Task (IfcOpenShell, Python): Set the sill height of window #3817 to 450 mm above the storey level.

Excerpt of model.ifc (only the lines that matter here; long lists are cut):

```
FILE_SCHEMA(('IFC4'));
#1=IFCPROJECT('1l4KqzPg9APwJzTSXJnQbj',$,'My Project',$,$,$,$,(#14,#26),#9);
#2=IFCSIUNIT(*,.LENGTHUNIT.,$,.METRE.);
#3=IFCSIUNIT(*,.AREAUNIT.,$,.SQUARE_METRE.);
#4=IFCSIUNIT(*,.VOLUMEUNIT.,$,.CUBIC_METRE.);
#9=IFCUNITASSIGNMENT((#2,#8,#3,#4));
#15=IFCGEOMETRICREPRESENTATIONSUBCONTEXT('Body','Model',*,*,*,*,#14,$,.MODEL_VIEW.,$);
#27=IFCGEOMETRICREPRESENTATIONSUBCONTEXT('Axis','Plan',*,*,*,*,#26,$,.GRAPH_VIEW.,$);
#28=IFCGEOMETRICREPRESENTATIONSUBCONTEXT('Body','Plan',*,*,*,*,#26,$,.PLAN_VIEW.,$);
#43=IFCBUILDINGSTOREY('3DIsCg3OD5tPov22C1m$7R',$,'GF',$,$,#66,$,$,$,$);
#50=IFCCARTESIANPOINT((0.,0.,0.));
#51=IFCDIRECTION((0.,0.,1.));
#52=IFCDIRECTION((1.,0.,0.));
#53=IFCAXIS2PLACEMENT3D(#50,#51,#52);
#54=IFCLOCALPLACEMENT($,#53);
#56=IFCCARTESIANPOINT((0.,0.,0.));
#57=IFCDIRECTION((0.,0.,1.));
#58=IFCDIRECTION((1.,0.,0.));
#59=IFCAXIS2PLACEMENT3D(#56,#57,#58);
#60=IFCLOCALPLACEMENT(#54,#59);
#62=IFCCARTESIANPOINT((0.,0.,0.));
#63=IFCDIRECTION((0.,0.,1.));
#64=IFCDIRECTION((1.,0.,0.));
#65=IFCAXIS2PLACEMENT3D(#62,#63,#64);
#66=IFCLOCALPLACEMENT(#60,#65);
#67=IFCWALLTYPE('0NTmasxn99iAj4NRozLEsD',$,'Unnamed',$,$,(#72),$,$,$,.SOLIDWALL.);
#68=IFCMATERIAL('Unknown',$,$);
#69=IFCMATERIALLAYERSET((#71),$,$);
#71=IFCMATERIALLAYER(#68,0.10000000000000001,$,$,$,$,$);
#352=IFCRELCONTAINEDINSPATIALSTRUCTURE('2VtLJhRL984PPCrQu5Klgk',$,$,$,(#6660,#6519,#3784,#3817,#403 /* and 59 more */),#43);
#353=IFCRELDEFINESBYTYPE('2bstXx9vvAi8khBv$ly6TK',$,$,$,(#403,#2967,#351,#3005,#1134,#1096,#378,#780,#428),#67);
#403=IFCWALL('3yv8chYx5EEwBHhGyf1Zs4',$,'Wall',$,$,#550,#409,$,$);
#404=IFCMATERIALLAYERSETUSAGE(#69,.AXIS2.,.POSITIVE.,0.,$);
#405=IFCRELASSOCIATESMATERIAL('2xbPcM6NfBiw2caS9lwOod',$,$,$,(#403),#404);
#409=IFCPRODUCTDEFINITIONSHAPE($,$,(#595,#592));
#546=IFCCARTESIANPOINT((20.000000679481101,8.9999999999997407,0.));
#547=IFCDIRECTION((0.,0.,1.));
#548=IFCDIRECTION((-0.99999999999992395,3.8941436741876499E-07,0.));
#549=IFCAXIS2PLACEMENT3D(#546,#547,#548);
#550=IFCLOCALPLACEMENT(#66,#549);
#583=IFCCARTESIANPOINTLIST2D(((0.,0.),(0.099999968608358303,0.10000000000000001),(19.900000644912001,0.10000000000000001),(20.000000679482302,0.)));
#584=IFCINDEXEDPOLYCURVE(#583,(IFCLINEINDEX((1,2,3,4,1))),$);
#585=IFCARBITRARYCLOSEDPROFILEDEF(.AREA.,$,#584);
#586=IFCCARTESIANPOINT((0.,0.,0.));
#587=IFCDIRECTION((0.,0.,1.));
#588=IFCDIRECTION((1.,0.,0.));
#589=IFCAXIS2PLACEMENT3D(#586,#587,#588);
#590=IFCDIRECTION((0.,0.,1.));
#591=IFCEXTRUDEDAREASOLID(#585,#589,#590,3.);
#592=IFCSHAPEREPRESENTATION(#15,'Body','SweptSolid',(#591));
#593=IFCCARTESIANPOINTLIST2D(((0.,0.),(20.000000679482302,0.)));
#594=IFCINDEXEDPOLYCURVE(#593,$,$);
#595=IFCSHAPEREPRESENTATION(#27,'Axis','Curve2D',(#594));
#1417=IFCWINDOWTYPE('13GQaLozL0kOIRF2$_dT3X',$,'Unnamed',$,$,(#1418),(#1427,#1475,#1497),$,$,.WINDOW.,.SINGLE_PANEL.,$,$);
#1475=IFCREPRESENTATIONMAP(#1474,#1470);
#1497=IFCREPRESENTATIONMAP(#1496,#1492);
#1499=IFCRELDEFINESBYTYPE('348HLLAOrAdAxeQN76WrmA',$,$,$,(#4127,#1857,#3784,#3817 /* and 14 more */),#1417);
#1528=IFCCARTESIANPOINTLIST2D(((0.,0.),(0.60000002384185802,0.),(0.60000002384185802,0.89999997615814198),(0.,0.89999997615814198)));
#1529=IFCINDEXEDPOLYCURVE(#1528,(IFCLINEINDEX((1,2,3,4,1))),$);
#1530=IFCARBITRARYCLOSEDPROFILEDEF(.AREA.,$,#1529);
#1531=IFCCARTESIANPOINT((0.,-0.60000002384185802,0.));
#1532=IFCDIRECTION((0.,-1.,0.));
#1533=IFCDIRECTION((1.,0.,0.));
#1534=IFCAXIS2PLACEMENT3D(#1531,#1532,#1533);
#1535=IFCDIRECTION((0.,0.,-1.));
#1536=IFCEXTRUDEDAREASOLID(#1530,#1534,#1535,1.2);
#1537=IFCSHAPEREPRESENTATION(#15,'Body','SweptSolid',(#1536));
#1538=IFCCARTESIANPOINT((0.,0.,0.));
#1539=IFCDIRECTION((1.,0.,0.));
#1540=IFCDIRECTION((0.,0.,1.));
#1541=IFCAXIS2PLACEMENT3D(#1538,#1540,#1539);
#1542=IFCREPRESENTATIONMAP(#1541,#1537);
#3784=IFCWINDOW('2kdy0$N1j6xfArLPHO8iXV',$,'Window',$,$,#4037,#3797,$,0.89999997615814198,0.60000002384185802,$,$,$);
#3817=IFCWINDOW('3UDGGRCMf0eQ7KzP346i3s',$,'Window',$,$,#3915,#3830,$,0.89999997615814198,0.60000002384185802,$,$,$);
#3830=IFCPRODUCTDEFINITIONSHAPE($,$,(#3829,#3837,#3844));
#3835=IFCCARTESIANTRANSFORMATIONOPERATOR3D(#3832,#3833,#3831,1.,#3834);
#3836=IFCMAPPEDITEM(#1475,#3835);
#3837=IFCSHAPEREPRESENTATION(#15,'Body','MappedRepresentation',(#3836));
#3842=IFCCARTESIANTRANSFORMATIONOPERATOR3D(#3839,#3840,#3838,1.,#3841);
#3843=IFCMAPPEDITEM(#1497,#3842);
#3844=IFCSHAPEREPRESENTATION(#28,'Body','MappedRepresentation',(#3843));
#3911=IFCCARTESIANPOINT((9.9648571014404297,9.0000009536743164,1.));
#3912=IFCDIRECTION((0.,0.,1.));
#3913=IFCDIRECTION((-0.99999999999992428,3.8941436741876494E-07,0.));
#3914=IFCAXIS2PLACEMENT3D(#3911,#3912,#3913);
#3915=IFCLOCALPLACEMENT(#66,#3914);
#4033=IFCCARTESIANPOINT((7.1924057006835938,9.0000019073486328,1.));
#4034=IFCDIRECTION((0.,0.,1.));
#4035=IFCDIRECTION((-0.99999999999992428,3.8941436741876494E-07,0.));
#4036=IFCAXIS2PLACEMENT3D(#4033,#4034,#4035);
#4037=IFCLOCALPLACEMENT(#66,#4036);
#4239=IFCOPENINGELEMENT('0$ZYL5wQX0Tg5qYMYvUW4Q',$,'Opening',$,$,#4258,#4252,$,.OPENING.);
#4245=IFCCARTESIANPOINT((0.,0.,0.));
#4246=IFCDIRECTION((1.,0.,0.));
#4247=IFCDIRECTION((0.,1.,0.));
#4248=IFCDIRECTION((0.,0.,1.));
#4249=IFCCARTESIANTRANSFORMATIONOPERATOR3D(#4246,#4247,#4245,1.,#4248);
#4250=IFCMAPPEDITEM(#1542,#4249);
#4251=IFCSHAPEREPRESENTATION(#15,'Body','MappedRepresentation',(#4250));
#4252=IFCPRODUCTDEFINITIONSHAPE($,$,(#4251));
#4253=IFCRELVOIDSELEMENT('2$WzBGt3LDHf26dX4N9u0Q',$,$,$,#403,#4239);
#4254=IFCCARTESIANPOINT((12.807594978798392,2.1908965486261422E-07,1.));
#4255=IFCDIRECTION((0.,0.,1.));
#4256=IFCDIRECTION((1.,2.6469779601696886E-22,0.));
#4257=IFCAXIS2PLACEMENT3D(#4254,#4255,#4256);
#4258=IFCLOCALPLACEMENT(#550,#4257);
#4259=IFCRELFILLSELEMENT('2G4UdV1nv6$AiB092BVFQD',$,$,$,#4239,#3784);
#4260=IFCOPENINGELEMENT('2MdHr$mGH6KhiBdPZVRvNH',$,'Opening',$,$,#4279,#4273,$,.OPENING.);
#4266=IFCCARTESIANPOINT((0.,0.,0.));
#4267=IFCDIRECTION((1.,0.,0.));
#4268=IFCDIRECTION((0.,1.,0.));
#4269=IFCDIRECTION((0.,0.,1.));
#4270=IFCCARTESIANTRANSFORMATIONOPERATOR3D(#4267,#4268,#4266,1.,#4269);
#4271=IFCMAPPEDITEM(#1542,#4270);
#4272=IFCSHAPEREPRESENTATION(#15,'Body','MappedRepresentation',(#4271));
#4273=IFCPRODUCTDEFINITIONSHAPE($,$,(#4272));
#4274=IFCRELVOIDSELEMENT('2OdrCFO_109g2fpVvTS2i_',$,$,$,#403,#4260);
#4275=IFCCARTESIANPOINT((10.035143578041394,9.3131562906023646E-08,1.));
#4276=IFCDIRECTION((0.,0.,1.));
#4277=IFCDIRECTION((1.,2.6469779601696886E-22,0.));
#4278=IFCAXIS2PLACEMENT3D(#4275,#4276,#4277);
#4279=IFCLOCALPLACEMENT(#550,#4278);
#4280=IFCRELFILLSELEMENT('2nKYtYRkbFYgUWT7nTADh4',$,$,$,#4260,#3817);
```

```python
import numpy as np
import ifcopenshell
import ifcopenshell.api.geometry
import ifcopenshell.geom
import ifcopenshell.util.element
import ifcopenshell.util.placement
import ifcopenshell.util.shape
import ifcopenshell.util.unit

model = ifcopenshell.open("model.ifc")
unit_scale = ifcopenshell.util.unit.calculate_unit_scale(model)

window = model.by_guid("3UDGGRCMf0eQ7KzP346i3s")
opening = window.FillsVoids[0].RelatingOpeningElement
storey = ifcopenshell.util.element.get_container(window, ifc_class="IfcBuildingStorey")
level = ifcopenshell.util.placement.get_local_placement(storey.ObjectPlacement)[2, 3]

# The opening's origin need not be at the sill, so measure its lowest point.
shape = ifcopenshell.geom.create_shape(ifcopenshell.geom.settings(), opening)
bottom = ifcopenshell.util.shape.get_shape_bottom_elevation(shape, shape.geometry) / unit_scale
dz = level + 0.45 / unit_scale - bottom

shift = np.array([0.0, 0.0, dz])
# The window is not placed relative to its opening, so move both.
for product in (opening, window):
    matrix = ifcopenshell.util.placement.get_local_placement(product.ObjectPlacement)
    matrix[:3, 3] += shift
    ifcopenshell.api.geometry.edit_object_placement(model, product=product, matrix=matrix, is_si=False)

print(f"moved by {dz * unit_scale:+.3f} m")

model.write("model_rev.ifc")
```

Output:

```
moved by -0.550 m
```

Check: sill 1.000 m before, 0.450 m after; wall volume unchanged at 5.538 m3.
